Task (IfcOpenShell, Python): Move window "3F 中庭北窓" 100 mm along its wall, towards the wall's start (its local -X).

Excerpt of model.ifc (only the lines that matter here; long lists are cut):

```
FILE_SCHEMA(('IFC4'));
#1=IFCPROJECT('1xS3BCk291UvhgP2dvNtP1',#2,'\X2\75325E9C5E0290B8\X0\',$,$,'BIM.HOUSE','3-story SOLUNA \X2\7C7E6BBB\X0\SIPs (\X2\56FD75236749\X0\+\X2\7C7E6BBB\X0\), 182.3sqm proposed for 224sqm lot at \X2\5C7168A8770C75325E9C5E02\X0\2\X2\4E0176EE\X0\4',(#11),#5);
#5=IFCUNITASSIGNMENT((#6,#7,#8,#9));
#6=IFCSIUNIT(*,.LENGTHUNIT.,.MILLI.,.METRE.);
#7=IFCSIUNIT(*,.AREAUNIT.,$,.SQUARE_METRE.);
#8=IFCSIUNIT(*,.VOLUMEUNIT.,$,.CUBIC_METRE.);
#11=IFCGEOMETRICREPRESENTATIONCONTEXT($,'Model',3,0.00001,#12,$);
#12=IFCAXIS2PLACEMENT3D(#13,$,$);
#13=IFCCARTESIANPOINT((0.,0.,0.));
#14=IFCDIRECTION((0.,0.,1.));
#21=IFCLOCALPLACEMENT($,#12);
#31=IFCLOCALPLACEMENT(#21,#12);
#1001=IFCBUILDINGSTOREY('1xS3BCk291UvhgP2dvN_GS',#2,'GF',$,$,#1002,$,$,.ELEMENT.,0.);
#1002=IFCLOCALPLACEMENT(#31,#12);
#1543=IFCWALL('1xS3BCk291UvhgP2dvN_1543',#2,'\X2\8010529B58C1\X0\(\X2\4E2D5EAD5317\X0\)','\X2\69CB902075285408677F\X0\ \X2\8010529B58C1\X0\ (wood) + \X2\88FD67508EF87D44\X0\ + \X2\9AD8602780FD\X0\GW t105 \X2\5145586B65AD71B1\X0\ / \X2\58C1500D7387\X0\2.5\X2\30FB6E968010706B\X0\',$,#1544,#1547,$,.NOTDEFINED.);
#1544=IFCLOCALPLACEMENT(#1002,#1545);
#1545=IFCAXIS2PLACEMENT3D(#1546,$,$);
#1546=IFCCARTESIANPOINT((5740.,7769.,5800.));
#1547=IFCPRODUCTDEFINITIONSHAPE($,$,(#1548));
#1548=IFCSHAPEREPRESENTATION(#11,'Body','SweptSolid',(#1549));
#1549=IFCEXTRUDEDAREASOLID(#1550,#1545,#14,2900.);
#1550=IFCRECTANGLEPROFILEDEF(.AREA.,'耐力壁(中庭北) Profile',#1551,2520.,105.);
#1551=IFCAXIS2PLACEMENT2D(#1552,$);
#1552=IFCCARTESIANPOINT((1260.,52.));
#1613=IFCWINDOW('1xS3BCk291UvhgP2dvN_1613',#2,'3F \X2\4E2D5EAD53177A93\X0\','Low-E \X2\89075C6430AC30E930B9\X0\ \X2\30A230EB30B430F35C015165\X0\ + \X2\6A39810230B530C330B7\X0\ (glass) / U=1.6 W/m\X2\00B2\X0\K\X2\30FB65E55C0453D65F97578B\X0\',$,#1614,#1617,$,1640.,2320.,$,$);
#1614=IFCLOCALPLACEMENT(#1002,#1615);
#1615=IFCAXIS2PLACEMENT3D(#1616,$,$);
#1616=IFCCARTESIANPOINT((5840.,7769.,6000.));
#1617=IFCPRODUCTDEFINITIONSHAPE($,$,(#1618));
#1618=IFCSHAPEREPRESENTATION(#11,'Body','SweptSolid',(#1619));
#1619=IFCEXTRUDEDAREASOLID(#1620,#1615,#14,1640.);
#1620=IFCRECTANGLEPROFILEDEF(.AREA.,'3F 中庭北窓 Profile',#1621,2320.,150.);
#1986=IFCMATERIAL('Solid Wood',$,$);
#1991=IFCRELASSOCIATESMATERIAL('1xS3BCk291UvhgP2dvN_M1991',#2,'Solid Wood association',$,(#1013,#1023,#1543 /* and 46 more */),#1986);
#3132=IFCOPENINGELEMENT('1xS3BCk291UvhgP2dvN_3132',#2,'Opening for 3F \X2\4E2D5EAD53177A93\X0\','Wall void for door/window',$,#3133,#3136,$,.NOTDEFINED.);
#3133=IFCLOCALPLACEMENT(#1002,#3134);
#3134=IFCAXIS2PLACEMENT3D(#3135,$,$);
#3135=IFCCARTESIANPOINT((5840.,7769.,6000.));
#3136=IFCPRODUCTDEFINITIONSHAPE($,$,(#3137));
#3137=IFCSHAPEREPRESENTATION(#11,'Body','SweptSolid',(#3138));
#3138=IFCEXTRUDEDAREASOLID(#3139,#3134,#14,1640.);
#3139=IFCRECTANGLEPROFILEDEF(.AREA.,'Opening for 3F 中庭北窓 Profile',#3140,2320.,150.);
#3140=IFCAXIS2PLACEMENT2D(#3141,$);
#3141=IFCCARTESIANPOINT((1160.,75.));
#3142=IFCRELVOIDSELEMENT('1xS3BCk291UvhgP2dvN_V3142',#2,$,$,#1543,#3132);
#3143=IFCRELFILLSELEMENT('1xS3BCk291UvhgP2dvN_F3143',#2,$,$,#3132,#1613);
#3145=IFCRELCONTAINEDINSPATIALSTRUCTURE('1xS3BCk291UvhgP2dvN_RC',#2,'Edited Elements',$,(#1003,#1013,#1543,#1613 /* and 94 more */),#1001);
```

```python
import ifcopenshell
import ifcopenshell.api.geometry
import ifcopenshell.util.placement
import ifcopenshell.util.unit

model = ifcopenshell.open("model.ifc")
unit_scale = ifcopenshell.util.unit.calculate_unit_scale(model)

window = model.by_guid("1xS3BCk291UvhgP2dvN_1613")
opening = window.FillsVoids[0].RelatingOpeningElement
wall = opening.VoidsElements[0].RelatingBuildingElement

wall_matrix = ifcopenshell.util.placement.get_local_placement(wall.ObjectPlacement)
shift = wall_matrix[:3, 0] * -0.1 / unit_scale
before = ifcopenshell.util.placement.get_local_placement(window.ObjectPlacement)[:3, 3].copy()

# The window is not placed relative to its opening, so move both.
for product in (opening, window):
    matrix = ifcopenshell.util.placement.get_local_placement(product.ObjectPlacement)
    matrix[:3, 3] += shift
    ifcopenshell.api.geometry.edit_object_placement(model, product=product, matrix=matrix, is_si=False)

after = ifcopenshell.util.placement.get_local_placement(window.ObjectPlacement)[:3, 3]
print("window moved by", (after - before).round(3) + 0.0)

model.write("model_updated.ifc")
```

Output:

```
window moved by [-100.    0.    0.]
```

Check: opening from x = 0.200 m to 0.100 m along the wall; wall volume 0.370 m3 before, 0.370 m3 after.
